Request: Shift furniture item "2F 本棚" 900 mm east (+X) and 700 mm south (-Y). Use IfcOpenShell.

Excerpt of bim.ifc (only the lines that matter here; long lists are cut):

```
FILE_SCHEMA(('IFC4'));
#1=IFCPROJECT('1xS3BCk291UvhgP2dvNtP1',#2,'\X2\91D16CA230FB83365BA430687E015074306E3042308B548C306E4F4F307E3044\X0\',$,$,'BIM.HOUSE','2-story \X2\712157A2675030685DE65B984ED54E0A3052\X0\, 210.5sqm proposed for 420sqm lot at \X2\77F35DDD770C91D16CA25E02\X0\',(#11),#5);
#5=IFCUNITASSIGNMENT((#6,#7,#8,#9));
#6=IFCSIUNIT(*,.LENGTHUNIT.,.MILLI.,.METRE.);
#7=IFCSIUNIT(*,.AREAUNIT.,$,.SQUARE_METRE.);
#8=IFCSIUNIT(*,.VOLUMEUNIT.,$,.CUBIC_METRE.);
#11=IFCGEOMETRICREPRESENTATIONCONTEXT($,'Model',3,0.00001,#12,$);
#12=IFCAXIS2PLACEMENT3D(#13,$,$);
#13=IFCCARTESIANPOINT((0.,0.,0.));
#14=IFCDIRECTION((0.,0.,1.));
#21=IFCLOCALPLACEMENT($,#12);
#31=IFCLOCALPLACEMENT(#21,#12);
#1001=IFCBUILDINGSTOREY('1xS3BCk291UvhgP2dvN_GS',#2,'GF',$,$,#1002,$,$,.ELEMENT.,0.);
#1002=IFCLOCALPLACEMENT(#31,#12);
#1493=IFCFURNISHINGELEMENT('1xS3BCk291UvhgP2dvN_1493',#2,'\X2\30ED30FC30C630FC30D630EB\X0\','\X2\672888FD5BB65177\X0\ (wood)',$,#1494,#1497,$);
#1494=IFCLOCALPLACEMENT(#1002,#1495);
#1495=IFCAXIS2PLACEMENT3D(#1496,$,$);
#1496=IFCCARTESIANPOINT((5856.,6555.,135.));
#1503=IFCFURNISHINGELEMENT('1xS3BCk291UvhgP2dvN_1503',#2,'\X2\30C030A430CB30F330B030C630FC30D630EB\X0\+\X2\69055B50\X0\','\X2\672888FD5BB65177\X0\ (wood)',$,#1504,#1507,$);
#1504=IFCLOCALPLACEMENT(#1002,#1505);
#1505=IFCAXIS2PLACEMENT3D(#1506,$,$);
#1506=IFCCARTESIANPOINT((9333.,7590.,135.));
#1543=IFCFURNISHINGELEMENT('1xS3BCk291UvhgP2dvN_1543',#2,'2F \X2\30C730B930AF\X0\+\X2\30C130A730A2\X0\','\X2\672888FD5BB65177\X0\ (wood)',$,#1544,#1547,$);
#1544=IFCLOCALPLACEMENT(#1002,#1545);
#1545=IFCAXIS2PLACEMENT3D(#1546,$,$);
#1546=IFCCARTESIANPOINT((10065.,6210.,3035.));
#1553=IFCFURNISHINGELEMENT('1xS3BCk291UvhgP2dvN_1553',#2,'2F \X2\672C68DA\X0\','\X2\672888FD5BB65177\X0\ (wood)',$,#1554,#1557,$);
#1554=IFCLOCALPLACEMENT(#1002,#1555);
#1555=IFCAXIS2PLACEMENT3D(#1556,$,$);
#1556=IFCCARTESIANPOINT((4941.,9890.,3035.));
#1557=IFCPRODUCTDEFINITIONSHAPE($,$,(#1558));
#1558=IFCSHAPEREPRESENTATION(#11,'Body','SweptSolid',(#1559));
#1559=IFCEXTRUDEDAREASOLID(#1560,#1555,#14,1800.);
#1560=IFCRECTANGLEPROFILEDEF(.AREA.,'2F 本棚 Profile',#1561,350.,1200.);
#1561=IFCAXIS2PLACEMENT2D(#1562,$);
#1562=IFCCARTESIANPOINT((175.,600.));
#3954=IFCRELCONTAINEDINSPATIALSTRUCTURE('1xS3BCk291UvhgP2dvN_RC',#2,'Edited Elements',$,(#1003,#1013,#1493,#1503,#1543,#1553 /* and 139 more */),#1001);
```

```python
import ifcopenshell
import ifcopenshell.api.geometry
import ifcopenshell.util.placement
import ifcopenshell.util.unit

model = ifcopenshell.open("bim.ifc")
unit_scale = ifcopenshell.util.unit.calculate_unit_scale(model)

item = model.by_guid("1xS3BCk291UvhgP2dvN_1553")
matrix = ifcopenshell.util.placement.get_local_placement(item.ObjectPlacement)
matrix[0, 3] += 0.9 / unit_scale
matrix[1, 3] -= 0.7 / unit_scale
ifcopenshell.api.geometry.edit_object_placement(model, product=item, matrix=matrix, is_si=False)

print(ifcopenshell.util.placement.get_local_placement(item.ObjectPlacement).round(3) + 0.0)

model.write("bim_edited.ifc")
```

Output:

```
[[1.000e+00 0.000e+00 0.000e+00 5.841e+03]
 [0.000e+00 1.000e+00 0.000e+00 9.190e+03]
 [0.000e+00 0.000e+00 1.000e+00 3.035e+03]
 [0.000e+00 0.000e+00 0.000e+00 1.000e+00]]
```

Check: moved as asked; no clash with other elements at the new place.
